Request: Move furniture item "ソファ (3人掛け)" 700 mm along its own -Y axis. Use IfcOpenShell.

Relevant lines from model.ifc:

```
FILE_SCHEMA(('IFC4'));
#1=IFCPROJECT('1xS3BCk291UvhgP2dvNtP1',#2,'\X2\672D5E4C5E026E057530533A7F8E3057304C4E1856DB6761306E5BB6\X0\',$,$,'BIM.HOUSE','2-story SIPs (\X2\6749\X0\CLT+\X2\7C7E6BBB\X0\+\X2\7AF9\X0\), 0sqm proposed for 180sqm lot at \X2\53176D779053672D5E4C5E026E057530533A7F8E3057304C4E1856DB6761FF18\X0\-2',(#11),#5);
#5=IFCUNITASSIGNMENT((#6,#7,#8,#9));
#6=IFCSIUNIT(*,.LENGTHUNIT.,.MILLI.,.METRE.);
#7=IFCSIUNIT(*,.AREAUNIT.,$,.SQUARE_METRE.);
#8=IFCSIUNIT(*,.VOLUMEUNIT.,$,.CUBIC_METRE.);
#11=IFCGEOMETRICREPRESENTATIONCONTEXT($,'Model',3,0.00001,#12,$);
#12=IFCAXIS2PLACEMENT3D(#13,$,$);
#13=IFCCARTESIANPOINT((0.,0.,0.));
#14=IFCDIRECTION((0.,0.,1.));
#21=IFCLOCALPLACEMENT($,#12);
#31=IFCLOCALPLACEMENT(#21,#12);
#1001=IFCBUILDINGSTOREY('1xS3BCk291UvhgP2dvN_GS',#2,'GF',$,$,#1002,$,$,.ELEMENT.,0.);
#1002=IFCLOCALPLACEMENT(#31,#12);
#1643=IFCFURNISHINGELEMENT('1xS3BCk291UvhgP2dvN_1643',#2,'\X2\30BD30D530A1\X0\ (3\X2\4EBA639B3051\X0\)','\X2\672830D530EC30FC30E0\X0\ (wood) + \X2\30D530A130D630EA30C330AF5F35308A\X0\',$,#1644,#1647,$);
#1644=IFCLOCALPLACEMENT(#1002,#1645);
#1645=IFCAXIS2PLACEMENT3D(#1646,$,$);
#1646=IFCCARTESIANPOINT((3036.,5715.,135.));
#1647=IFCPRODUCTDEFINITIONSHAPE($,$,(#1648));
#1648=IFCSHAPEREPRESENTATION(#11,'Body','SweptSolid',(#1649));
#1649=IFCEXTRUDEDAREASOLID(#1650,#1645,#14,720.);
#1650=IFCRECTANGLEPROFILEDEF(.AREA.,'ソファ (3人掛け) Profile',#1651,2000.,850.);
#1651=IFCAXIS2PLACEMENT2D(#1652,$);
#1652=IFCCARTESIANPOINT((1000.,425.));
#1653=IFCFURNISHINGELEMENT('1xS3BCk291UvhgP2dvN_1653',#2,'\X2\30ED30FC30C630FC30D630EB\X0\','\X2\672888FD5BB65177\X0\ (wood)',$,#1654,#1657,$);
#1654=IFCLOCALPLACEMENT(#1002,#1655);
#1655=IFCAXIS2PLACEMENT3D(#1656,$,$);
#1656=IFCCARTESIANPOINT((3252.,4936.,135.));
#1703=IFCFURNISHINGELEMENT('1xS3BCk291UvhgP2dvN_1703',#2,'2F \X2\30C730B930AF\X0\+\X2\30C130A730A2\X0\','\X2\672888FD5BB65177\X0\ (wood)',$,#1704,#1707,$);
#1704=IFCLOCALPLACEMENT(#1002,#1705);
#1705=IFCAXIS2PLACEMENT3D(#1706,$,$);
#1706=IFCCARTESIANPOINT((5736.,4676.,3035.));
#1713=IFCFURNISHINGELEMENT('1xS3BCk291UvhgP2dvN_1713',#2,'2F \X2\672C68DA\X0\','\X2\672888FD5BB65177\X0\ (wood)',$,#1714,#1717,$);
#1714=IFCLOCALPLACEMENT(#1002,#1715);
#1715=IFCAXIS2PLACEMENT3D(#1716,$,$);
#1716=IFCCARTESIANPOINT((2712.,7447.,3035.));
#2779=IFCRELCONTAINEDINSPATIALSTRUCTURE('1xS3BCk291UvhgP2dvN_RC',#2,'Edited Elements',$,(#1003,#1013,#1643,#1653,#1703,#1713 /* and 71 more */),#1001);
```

```python
import ifcopenshell
import ifcopenshell.api.geometry
import ifcopenshell.util.placement

model = ifcopenshell.open("model.ifc")

item = model.by_id(1643)
matrix = ifcopenshell.util.placement.get_local_placement(item.ObjectPlacement)
matrix[:3, 3] -= matrix[:3, 1] * 700.0
ifcopenshell.api.geometry.edit_object_placement(model, product=item, matrix=matrix, is_si=False)

print(ifcopenshell.util.placement.get_local_placement(item.ObjectPlacement).round(3) + 0.0)

model.write("model_v2.ifc")
```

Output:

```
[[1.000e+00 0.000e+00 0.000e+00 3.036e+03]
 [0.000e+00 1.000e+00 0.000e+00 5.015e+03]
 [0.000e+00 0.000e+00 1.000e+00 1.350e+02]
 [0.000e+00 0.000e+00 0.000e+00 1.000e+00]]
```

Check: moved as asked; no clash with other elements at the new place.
